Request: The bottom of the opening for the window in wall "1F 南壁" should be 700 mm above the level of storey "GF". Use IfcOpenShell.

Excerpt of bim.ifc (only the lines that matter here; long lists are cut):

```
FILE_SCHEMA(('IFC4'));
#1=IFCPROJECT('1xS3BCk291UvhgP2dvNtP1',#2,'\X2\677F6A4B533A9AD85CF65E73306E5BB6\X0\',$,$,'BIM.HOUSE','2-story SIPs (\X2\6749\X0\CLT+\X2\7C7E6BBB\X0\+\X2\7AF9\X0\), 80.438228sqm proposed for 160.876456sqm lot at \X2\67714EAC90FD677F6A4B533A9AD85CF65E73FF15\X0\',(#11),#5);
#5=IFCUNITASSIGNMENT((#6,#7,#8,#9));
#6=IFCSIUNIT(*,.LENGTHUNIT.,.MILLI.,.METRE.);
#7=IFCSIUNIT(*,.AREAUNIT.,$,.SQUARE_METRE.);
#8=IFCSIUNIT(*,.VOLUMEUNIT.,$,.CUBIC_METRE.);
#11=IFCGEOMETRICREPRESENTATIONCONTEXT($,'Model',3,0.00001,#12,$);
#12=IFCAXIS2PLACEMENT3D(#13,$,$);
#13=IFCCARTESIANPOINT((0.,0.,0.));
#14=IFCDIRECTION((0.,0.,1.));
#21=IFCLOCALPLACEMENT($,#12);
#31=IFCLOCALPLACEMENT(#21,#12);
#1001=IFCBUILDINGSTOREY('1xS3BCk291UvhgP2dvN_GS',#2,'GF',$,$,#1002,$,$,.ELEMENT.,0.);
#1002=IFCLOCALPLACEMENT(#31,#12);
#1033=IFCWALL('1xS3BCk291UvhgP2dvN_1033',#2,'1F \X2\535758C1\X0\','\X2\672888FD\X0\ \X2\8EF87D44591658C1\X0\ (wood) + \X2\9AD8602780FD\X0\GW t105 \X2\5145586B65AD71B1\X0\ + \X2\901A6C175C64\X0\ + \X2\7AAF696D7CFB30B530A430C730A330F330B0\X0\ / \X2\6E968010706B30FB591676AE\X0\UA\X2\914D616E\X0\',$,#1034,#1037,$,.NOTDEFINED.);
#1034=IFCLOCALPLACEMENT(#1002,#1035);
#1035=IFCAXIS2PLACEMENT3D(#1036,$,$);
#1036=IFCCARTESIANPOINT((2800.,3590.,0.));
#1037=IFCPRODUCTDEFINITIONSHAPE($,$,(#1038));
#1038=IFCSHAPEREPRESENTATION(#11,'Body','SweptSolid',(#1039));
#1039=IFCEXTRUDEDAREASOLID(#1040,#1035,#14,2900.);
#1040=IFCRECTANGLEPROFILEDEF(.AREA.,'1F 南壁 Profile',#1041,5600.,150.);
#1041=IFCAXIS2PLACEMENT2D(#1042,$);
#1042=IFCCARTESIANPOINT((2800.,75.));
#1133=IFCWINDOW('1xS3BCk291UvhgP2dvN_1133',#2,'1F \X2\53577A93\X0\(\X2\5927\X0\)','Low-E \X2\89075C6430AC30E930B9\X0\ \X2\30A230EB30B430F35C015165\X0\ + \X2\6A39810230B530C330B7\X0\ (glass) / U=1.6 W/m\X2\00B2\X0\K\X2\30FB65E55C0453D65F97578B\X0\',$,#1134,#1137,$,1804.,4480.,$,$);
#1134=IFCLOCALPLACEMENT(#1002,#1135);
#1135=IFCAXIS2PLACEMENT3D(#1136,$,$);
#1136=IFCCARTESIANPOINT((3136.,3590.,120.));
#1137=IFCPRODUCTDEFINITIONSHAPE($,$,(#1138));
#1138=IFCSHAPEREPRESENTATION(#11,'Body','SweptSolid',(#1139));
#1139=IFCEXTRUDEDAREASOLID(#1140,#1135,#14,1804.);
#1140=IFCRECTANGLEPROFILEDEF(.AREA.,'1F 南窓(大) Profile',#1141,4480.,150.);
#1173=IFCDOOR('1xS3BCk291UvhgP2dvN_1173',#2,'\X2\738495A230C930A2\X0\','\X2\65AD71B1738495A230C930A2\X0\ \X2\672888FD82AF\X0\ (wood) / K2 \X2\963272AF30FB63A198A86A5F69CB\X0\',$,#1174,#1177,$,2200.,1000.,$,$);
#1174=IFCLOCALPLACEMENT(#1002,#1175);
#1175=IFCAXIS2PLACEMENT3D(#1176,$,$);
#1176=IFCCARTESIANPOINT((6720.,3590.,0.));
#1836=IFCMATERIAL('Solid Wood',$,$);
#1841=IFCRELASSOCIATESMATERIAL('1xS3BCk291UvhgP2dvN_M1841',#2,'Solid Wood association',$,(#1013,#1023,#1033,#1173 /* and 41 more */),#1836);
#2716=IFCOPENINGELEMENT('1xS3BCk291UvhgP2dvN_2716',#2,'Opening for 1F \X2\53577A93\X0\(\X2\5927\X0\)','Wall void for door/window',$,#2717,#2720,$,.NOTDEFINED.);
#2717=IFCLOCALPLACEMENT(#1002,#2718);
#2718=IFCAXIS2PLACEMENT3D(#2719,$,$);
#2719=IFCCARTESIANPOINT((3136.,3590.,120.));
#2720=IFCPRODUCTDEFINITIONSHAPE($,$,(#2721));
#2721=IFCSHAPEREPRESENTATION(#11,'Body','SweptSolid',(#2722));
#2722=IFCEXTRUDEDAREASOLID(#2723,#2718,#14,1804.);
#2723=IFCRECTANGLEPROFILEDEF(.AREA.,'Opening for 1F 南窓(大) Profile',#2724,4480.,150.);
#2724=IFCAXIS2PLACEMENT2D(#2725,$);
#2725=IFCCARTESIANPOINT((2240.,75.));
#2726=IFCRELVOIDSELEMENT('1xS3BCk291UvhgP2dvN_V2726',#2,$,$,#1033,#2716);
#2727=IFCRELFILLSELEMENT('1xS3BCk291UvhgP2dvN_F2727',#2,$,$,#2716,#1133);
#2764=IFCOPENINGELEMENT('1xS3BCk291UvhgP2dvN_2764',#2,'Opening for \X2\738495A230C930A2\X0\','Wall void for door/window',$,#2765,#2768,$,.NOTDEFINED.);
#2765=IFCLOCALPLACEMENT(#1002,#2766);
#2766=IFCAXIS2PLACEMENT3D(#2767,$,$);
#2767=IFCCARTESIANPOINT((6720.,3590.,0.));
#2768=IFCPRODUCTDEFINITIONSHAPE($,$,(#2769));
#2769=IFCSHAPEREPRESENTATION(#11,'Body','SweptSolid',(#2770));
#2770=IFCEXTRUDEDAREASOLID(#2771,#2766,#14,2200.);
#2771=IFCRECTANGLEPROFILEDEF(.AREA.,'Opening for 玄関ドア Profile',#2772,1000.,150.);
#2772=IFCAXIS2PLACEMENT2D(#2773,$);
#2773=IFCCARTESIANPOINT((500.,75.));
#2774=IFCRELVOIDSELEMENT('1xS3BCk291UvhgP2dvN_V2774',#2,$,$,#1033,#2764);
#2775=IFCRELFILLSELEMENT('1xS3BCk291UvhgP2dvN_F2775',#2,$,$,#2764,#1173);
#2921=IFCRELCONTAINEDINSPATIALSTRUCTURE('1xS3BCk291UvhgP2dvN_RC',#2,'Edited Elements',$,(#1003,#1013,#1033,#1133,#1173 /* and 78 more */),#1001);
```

```python
import numpy as np
import ifcopenshell
import ifcopenshell.api.geometry
import ifcopenshell.geom
import ifcopenshell.util.element
import ifcopenshell.util.placement
import ifcopenshell.util.shape
import ifcopenshell.util.unit

model = ifcopenshell.open("bim.ifc")
unit_scale = ifcopenshell.util.unit.calculate_unit_scale(model)

window = model.by_guid("1xS3BCk291UvhgP2dvN_1133")
opening = window.FillsVoids[0].RelatingOpeningElement
storey = ifcopenshell.util.element.get_container(window, ifc_class="IfcBuildingStorey")
level = ifcopenshell.util.placement.get_local_placement(storey.ObjectPlacement)[2, 3]

# The opening's origin need not be at the sill, so measure its lowest point.
shape = ifcopenshell.geom.create_shape(ifcopenshell.geom.settings(), opening)
bottom = ifcopenshell.util.shape.get_shape_bottom_elevation(shape, shape.geometry) / unit_scale
dz = level + 0.7 / unit_scale - bottom

shift = np.array([0.0, 0.0, dz])
# The window is not placed relative to its opening, so move both.
for product in (opening, window):
    matrix = ifcopenshell.util.placement.get_local_placement(product.ObjectPlacement)
    matrix[:3, 3] += shift
    ifcopenshell.api.geometry.edit_object_placement(model, product=product, matrix=matrix, is_si=False)

print(f"moved by {dz * unit_scale:+.3f} m")

model.write("bim_v2.ifc")
```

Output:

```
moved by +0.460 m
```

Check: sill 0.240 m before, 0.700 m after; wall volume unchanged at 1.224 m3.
